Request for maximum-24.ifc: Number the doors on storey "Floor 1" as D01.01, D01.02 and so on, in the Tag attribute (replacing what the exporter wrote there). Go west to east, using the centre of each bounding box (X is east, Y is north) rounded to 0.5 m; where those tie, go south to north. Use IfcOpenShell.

First a look at what the model holds.

```python
import ifcopenshell
import ifcopenshell.util.element
import ifcopenshell.util.placement

model = ifcopenshell.open("maximum-24.ifc")
print(model.schema)
storey = next(s for s in model.by_type("IfcBuildingStorey") if s.Name == "Floor 1")
doors = [e for e in ifcopenshell.util.element.get_decomposition(storey) if e.is_a("IfcDoor")]
for e in sorted(doors, key=lambda e: e.id()):
    origin = ifcopenshell.util.placement.get_local_placement(e.ObjectPlacement)[:3, 3]
    print(e.id(), e.Tag, e.Name, origin.round(2) + 0.0, sep=" | ")
```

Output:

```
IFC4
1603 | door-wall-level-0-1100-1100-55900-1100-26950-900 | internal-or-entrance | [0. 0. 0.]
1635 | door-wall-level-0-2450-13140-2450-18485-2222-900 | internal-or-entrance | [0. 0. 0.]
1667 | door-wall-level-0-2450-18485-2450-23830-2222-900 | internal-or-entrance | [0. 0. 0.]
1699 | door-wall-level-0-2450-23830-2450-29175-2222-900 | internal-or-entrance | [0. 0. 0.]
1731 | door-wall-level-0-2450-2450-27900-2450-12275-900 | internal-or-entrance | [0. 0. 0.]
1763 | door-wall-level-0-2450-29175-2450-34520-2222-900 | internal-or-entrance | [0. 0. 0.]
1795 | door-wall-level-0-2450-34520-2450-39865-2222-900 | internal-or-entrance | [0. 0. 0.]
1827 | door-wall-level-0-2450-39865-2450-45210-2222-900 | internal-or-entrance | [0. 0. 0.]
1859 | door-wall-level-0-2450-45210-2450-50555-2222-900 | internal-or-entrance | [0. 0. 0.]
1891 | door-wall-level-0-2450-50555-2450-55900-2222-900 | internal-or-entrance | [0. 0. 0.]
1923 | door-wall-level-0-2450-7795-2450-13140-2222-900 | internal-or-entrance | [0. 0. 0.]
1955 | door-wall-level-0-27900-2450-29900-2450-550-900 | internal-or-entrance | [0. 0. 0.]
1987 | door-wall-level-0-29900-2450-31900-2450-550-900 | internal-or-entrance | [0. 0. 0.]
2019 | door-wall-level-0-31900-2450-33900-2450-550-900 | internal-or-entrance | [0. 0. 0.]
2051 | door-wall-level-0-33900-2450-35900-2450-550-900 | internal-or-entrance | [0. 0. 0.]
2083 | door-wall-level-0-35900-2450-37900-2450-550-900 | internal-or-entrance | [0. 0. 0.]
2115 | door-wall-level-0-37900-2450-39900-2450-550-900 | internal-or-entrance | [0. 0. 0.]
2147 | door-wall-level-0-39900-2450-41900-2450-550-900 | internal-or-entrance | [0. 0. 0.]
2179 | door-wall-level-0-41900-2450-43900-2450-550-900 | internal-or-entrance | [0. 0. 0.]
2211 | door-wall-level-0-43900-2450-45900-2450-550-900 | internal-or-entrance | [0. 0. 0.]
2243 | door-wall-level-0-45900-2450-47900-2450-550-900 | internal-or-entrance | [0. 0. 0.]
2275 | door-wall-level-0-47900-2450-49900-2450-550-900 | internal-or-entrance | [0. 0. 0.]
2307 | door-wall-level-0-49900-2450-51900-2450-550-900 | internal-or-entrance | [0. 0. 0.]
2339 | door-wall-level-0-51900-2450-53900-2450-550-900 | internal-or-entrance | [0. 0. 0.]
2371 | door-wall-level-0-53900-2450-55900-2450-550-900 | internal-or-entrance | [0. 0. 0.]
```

```python
import ifcopenshell
import ifcopenshell.geom
import ifcopenshell.util.element
import ifcopenshell.util.shape

model = ifcopenshell.open("maximum-24.ifc")
settings = ifcopenshell.geom.settings()
settings.set("use-world-coords", True)


def centre(element):
    shape = ifcopenshell.geom.create_shape(settings, element)
    return ifcopenshell.util.shape.get_bbox_centroid(shape.geometry)


storey = next(s for s in model.by_type("IfcBuildingStorey") if s.Name == "Floor 1")
doors = [e for e in ifcopenshell.util.element.get_decomposition(storey) if e.is_a("IfcDoor")]

# Insertion points can sit at a corner or the storey origin, so sort by the geometry (in metres).
centres = {e: centre(e) for e in doors}
doors.sort(key=lambda e: (round(centres[e][0] / 0.5), centres[e][1]))

for i, e in enumerate(doors, start=1):
    number = f"D01.{i:02d}"
    e.Tag = number
    print(e.id(), number)

model.write("maximum-24-out.ifc")
```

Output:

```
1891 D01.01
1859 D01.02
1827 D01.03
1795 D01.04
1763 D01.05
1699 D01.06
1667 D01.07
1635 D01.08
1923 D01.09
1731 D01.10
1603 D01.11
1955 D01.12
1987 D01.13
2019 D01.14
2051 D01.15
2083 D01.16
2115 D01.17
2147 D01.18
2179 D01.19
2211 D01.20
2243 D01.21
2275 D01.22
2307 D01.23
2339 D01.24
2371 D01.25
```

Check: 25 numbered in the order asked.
